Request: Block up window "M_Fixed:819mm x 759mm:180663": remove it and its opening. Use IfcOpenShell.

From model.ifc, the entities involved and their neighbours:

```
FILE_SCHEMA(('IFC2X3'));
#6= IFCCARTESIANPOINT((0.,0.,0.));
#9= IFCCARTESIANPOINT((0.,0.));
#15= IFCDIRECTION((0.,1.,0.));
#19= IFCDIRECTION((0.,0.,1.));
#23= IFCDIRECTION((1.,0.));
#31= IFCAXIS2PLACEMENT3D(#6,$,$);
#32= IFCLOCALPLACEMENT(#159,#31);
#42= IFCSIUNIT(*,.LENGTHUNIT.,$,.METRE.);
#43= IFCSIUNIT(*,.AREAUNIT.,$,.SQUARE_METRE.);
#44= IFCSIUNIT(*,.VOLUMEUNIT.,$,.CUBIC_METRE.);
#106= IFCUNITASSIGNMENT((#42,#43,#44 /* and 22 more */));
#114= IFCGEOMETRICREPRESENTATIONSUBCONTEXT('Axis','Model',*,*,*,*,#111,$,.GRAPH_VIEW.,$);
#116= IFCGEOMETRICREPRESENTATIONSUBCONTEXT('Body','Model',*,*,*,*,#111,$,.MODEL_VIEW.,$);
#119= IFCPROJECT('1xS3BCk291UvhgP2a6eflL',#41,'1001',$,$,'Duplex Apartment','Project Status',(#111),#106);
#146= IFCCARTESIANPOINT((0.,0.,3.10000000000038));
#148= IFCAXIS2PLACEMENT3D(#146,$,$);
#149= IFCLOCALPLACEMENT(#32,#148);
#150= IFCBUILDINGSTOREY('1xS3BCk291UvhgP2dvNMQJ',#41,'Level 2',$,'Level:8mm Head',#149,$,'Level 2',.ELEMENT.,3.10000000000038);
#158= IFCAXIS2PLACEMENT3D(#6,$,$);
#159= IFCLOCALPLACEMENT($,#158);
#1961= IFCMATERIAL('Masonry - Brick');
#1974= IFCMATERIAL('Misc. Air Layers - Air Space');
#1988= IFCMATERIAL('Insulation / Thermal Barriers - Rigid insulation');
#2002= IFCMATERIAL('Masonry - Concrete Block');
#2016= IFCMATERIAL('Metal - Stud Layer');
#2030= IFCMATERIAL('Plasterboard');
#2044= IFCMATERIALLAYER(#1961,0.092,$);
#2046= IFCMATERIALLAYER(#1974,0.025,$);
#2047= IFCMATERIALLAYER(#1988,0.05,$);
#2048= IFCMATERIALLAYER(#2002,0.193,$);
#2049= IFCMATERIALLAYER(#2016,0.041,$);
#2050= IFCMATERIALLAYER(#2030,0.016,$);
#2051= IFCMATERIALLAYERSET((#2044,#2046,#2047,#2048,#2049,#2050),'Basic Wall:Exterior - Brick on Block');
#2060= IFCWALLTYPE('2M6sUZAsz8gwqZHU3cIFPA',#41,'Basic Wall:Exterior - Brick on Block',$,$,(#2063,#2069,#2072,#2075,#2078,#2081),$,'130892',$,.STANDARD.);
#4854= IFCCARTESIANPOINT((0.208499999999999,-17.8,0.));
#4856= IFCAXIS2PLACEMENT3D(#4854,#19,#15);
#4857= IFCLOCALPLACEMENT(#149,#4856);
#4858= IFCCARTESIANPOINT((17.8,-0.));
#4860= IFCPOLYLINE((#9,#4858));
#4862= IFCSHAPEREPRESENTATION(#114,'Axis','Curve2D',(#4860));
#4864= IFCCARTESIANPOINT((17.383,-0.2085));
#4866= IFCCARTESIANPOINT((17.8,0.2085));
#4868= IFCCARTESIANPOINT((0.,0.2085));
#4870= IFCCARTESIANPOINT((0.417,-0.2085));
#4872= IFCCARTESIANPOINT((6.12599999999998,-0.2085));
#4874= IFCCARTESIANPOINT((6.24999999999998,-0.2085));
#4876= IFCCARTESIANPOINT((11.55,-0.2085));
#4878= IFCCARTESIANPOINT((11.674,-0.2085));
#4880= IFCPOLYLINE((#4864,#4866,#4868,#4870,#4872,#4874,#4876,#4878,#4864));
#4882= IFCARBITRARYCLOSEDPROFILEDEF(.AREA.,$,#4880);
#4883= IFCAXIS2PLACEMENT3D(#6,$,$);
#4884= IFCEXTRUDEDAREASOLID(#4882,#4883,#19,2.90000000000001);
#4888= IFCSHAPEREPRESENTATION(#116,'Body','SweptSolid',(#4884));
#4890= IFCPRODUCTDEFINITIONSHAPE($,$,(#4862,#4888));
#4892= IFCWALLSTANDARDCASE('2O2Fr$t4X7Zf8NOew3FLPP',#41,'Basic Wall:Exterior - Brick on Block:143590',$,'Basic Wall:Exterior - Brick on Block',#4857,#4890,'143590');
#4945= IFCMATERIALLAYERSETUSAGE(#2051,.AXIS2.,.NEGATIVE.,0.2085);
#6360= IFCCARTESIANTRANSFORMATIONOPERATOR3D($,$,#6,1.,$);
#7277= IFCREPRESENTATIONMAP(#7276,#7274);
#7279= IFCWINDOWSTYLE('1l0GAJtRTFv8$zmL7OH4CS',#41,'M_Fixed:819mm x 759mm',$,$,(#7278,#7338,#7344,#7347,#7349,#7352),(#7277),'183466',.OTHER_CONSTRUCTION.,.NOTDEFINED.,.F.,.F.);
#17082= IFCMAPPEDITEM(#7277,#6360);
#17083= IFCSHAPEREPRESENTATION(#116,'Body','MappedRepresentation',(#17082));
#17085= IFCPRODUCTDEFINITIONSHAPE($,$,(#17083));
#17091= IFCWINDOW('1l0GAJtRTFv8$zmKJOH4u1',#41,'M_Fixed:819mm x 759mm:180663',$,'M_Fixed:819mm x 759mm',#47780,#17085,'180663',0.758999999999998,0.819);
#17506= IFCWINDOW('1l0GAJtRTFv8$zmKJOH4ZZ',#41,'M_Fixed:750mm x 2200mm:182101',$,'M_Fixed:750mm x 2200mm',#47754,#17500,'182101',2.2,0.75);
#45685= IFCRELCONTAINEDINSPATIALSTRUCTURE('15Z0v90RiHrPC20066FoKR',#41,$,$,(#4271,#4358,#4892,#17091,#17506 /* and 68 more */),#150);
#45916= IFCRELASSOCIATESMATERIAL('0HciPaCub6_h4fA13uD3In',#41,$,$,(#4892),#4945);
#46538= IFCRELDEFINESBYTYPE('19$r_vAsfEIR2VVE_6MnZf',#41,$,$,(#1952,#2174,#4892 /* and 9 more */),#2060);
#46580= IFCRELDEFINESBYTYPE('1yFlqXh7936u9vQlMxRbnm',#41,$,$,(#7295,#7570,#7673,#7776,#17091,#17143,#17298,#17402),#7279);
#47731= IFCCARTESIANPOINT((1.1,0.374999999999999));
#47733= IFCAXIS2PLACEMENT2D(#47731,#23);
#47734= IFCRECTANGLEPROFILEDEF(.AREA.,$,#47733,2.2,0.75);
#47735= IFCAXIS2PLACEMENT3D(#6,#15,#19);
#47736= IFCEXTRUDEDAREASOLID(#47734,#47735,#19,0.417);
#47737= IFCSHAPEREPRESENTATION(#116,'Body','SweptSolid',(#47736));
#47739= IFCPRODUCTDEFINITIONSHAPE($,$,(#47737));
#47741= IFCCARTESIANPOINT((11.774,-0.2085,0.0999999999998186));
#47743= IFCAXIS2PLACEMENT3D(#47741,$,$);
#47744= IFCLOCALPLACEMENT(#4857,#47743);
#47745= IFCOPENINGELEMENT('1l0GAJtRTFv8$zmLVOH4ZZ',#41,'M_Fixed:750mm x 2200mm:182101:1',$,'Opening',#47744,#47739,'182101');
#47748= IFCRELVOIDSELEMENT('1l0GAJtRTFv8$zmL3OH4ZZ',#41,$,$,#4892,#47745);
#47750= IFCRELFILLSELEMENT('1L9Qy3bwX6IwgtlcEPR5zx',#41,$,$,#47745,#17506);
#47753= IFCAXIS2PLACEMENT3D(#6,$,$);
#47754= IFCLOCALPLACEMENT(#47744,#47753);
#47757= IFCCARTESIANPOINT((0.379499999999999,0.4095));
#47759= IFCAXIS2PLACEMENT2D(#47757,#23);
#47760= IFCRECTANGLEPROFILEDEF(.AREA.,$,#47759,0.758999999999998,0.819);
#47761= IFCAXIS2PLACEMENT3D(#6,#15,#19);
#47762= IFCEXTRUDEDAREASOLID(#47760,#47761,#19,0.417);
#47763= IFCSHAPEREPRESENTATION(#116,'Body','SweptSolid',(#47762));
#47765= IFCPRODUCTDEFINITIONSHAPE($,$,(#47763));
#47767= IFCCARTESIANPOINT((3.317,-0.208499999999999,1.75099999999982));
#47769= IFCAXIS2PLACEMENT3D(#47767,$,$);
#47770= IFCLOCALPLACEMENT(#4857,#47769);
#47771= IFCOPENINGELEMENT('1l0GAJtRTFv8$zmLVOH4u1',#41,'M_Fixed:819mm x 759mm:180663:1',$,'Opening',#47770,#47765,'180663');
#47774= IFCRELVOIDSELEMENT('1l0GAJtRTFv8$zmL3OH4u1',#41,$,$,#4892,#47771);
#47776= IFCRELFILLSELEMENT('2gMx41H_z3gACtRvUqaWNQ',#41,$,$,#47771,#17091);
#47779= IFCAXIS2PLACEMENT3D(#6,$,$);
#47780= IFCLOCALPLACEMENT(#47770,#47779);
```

```python
import ifcopenshell
import ifcopenshell.api.feature
import ifcopenshell.api.root
import ifcopenshell.geom
import ifcopenshell.util.shape

model = ifcopenshell.open("model.ifc")
settings = ifcopenshell.geom.settings()


def volume(element):
    """Net volume in cubic metres, openings subtracted."""
    shape = ifcopenshell.geom.create_shape(settings, element)
    return ifcopenshell.util.shape.get_volume(shape.geometry)


window = model.by_id(17091)
opening = window.FillsVoids[0].RelatingOpeningElement
wall = opening.VoidsElements[0].RelatingBuildingElement
before = volume(wall)

ifcopenshell.api.root.remove_product(model, product=window)
ifcopenshell.api.feature.remove_feature(model, feature=opening)

after = volume(wall)

print(f"wall volume {before:.3f} -> {after:.3f} m3")

model.write("model_edited.ifc")
```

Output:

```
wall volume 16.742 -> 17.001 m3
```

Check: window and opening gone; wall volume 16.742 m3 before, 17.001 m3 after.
